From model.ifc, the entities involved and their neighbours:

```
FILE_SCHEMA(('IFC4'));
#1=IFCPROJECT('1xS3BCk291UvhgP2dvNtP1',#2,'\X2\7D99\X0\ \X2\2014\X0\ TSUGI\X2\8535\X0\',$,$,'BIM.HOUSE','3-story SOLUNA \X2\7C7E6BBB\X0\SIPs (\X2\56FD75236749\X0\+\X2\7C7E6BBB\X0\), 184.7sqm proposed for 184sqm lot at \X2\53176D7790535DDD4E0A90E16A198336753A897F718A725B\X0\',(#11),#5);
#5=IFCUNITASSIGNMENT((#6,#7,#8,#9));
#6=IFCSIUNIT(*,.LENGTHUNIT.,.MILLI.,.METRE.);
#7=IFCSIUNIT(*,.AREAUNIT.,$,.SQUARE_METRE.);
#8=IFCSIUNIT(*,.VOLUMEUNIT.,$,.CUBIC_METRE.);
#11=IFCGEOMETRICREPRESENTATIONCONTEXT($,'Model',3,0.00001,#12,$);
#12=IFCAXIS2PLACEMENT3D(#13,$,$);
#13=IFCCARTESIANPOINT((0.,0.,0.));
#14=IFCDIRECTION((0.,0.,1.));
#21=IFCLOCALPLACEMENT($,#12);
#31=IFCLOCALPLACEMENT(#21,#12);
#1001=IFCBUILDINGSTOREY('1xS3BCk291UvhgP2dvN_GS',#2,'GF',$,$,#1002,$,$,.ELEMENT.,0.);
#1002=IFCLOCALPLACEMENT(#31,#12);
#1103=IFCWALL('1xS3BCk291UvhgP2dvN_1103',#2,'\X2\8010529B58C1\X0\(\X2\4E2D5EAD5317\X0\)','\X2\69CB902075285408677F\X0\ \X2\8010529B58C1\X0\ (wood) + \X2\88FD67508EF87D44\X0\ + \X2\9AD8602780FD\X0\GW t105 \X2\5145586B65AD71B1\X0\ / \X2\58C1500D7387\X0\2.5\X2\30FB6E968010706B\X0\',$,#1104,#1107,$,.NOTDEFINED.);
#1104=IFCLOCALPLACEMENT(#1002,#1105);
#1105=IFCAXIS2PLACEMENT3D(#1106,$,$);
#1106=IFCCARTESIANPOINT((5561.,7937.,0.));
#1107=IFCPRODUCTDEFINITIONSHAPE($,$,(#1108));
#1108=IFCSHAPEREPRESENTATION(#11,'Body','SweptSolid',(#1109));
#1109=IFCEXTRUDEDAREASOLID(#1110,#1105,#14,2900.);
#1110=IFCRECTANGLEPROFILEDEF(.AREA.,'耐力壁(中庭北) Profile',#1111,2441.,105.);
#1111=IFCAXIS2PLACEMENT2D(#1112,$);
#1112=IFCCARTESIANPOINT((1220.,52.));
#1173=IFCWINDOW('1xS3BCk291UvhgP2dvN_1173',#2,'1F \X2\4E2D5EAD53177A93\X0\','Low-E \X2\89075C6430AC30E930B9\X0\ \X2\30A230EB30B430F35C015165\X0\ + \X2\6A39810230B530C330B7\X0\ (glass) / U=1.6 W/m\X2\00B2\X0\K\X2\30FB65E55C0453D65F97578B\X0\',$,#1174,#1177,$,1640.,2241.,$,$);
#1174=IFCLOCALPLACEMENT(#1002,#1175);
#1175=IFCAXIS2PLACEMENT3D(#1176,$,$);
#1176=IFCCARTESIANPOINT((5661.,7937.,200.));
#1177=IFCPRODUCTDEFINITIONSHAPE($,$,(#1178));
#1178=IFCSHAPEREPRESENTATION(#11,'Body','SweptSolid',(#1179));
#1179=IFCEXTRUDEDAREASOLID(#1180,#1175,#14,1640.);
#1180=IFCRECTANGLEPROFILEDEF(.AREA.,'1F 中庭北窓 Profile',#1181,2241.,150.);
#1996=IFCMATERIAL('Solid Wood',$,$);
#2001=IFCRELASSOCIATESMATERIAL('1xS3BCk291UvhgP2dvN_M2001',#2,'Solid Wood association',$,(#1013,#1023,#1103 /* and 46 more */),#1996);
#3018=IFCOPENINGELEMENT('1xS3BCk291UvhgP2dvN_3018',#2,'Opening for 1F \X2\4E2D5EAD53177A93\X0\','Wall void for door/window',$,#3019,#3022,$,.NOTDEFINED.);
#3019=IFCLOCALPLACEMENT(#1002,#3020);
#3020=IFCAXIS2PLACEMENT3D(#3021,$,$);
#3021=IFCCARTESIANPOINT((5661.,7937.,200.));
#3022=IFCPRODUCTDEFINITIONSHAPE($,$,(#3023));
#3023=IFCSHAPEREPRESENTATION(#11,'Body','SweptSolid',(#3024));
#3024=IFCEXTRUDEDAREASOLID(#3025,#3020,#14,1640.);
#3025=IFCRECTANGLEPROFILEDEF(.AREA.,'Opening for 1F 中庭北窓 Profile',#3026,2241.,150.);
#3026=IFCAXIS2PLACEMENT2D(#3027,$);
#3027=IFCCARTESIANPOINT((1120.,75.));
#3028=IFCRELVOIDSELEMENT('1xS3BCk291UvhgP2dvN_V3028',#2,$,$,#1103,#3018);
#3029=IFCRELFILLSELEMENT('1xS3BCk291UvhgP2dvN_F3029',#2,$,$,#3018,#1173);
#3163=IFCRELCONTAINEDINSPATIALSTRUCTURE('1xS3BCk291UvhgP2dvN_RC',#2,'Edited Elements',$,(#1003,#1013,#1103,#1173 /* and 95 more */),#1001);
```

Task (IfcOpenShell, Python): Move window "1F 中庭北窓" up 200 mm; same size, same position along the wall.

```python
import numpy as np
import ifcopenshell
import ifcopenshell.api.geometry
import ifcopenshell.util.placement
import ifcopenshell.util.unit

model = ifcopenshell.open("model.ifc")
unit_scale = ifcopenshell.util.unit.calculate_unit_scale(model)

window = model.by_guid("1xS3BCk291UvhgP2dvN_1173")
opening = window.FillsVoids[0].RelatingOpeningElement
dz = 200.0

shift = np.array([0.0, 0.0, dz])
# The window is not placed relative to its opening, so move both.
for product in (opening, window):
    matrix = ifcopenshell.util.placement.get_local_placement(product.ObjectPlacement)
    matrix[:3, 3] += shift
    ifcopenshell.api.geometry.edit_object_placement(model, product=product, matrix=matrix, is_si=False)

print(f"moved by {dz * unit_scale:+.3f} m")

model.write("model_updated.ifc")
```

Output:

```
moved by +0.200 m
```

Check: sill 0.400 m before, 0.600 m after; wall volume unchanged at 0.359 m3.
